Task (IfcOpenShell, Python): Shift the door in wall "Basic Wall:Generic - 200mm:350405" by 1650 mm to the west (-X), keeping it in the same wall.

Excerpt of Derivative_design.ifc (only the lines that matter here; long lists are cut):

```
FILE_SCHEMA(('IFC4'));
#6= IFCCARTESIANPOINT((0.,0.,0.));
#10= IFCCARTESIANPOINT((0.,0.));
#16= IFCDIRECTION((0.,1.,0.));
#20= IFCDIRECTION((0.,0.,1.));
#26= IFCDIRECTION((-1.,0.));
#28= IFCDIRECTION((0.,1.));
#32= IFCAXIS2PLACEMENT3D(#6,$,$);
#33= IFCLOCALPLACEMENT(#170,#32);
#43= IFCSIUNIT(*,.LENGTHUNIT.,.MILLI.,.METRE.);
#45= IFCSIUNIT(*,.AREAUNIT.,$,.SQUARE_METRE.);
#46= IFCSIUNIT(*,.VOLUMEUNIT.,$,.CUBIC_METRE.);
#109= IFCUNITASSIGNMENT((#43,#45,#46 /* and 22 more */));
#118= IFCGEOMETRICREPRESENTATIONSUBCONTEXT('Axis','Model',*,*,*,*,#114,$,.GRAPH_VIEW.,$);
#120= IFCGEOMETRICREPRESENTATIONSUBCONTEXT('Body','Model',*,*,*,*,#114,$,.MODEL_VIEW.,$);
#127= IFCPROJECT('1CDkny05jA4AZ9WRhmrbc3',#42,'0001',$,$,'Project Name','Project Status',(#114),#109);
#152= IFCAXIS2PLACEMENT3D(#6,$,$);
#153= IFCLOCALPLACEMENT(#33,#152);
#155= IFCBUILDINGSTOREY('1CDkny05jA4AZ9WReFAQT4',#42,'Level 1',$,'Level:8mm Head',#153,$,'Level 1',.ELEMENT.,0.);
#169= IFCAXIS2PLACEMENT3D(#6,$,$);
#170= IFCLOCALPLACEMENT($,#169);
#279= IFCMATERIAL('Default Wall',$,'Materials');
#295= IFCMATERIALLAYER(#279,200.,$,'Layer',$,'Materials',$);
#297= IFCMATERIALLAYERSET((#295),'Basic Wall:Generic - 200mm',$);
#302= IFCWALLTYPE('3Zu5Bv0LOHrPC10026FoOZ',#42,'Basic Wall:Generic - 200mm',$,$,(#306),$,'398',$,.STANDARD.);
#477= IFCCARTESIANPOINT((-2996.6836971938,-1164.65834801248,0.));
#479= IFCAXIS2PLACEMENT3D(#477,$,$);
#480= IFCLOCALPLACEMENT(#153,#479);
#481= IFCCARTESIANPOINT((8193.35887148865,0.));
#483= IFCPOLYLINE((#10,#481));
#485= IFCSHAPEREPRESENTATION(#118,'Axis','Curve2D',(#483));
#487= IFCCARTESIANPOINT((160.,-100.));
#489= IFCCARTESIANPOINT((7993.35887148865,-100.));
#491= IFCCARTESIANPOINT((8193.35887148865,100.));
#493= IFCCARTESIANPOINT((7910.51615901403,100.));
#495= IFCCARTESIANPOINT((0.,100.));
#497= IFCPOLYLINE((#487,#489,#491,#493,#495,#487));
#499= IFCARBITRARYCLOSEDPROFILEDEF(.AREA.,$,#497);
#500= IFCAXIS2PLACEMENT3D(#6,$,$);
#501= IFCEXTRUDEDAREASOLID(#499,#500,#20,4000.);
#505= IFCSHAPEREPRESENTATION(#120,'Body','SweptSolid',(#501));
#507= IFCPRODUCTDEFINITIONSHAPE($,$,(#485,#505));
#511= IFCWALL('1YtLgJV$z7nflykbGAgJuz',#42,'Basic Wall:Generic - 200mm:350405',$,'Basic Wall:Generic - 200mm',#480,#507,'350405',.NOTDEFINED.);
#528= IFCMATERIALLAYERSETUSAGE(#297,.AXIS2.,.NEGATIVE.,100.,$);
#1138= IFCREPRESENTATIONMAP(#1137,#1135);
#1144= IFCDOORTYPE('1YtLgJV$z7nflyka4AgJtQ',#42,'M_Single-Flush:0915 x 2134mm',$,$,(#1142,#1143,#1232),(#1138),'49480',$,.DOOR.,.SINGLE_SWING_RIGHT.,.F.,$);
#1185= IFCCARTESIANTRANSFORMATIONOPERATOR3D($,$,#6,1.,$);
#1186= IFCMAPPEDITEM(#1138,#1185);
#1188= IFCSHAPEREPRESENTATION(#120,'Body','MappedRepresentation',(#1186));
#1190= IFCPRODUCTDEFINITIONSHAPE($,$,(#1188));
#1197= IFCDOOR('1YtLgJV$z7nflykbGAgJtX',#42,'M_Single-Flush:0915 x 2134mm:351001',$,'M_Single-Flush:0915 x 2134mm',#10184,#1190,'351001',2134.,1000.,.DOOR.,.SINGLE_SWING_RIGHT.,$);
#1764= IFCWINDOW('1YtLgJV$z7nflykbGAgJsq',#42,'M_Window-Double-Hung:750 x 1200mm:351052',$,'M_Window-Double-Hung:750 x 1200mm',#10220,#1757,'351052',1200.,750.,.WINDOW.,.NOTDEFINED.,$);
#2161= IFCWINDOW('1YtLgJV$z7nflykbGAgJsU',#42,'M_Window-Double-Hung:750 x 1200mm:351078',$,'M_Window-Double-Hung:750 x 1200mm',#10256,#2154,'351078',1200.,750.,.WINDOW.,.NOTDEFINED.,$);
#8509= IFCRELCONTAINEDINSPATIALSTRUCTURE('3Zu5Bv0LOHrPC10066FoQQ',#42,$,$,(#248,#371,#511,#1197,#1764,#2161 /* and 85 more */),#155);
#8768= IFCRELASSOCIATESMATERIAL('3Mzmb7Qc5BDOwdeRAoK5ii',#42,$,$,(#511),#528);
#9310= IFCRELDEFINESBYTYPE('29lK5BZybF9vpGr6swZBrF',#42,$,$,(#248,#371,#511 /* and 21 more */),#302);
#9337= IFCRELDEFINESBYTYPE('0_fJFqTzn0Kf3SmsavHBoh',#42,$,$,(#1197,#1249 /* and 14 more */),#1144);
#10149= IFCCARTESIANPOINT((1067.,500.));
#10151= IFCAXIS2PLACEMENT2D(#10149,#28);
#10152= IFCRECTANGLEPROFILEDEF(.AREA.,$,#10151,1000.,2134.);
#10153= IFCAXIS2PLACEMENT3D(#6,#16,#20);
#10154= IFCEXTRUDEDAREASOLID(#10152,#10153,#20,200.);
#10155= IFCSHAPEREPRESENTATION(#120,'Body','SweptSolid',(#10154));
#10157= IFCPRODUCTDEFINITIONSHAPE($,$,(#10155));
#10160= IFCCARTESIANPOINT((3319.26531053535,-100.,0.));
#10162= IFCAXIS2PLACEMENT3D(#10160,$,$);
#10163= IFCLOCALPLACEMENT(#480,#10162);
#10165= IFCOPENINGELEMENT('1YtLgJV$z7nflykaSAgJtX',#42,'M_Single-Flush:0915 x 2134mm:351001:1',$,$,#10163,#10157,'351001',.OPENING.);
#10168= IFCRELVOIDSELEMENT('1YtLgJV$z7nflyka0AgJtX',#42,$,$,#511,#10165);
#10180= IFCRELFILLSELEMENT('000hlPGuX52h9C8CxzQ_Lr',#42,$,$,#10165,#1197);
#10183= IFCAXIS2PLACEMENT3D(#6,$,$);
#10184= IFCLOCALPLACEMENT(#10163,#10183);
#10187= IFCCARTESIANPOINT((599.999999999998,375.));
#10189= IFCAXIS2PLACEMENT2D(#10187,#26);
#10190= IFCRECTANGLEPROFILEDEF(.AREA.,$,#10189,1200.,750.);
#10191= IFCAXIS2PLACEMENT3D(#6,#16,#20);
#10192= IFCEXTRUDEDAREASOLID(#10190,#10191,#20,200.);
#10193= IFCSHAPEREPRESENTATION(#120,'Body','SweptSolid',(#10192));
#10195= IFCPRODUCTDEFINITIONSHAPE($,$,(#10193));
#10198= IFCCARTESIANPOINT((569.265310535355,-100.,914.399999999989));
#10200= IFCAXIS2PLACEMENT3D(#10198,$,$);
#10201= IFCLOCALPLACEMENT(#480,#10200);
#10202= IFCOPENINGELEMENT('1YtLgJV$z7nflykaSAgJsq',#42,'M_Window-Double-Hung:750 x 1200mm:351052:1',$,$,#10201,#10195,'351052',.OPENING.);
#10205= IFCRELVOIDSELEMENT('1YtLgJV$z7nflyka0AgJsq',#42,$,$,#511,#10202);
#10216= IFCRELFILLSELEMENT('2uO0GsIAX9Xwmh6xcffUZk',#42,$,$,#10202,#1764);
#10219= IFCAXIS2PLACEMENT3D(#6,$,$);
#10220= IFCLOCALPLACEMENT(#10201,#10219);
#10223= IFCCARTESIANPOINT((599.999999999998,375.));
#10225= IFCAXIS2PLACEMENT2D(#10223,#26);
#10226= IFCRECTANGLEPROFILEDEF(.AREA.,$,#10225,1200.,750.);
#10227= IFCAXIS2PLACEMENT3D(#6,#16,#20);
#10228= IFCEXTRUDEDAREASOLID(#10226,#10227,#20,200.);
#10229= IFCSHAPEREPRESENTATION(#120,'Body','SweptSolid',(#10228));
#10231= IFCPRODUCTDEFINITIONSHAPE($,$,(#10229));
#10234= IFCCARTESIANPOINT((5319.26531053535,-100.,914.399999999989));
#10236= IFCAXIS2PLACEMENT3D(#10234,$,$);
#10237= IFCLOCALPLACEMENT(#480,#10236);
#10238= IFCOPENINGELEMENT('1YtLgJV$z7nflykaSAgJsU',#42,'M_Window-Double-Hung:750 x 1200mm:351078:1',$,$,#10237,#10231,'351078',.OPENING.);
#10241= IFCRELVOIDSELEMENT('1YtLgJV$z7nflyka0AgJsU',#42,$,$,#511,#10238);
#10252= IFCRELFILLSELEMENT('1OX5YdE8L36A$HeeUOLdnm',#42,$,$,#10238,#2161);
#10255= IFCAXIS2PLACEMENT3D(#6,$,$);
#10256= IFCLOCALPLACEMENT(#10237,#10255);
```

```python
import ifcopenshell
import ifcopenshell.api.geometry
import ifcopenshell.util.placement

model = ifcopenshell.open("Derivative_design.ifc")

door = model.by_guid("1YtLgJV$z7nflykbGAgJtX")
opening = door.FillsVoids[0].RelatingOpeningElement
wall = opening.VoidsElements[0].RelatingBuildingElement

wall_matrix = ifcopenshell.util.placement.get_local_placement(wall.ObjectPlacement)
shift = wall_matrix[:3, 0] * -1650.0
before = ifcopenshell.util.placement.get_local_placement(door.ObjectPlacement)[:3, 3].copy()

# The door is placed relative to its opening, so it follows when the opening moves.
matrix = ifcopenshell.util.placement.get_local_placement(opening.ObjectPlacement)
matrix[:3, 3] += shift
ifcopenshell.api.geometry.edit_object_placement(
    model, product=opening, matrix=matrix, is_si=False, should_transform_children=True
)

after = ifcopenshell.util.placement.get_local_placement(door.ObjectPlacement)[:3, 3]
print("door moved by", (after - before).round(3) + 0.0)

model.write("Derivative_design_edited.ifc")
```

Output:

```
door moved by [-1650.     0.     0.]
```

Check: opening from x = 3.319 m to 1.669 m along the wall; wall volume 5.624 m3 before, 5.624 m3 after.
